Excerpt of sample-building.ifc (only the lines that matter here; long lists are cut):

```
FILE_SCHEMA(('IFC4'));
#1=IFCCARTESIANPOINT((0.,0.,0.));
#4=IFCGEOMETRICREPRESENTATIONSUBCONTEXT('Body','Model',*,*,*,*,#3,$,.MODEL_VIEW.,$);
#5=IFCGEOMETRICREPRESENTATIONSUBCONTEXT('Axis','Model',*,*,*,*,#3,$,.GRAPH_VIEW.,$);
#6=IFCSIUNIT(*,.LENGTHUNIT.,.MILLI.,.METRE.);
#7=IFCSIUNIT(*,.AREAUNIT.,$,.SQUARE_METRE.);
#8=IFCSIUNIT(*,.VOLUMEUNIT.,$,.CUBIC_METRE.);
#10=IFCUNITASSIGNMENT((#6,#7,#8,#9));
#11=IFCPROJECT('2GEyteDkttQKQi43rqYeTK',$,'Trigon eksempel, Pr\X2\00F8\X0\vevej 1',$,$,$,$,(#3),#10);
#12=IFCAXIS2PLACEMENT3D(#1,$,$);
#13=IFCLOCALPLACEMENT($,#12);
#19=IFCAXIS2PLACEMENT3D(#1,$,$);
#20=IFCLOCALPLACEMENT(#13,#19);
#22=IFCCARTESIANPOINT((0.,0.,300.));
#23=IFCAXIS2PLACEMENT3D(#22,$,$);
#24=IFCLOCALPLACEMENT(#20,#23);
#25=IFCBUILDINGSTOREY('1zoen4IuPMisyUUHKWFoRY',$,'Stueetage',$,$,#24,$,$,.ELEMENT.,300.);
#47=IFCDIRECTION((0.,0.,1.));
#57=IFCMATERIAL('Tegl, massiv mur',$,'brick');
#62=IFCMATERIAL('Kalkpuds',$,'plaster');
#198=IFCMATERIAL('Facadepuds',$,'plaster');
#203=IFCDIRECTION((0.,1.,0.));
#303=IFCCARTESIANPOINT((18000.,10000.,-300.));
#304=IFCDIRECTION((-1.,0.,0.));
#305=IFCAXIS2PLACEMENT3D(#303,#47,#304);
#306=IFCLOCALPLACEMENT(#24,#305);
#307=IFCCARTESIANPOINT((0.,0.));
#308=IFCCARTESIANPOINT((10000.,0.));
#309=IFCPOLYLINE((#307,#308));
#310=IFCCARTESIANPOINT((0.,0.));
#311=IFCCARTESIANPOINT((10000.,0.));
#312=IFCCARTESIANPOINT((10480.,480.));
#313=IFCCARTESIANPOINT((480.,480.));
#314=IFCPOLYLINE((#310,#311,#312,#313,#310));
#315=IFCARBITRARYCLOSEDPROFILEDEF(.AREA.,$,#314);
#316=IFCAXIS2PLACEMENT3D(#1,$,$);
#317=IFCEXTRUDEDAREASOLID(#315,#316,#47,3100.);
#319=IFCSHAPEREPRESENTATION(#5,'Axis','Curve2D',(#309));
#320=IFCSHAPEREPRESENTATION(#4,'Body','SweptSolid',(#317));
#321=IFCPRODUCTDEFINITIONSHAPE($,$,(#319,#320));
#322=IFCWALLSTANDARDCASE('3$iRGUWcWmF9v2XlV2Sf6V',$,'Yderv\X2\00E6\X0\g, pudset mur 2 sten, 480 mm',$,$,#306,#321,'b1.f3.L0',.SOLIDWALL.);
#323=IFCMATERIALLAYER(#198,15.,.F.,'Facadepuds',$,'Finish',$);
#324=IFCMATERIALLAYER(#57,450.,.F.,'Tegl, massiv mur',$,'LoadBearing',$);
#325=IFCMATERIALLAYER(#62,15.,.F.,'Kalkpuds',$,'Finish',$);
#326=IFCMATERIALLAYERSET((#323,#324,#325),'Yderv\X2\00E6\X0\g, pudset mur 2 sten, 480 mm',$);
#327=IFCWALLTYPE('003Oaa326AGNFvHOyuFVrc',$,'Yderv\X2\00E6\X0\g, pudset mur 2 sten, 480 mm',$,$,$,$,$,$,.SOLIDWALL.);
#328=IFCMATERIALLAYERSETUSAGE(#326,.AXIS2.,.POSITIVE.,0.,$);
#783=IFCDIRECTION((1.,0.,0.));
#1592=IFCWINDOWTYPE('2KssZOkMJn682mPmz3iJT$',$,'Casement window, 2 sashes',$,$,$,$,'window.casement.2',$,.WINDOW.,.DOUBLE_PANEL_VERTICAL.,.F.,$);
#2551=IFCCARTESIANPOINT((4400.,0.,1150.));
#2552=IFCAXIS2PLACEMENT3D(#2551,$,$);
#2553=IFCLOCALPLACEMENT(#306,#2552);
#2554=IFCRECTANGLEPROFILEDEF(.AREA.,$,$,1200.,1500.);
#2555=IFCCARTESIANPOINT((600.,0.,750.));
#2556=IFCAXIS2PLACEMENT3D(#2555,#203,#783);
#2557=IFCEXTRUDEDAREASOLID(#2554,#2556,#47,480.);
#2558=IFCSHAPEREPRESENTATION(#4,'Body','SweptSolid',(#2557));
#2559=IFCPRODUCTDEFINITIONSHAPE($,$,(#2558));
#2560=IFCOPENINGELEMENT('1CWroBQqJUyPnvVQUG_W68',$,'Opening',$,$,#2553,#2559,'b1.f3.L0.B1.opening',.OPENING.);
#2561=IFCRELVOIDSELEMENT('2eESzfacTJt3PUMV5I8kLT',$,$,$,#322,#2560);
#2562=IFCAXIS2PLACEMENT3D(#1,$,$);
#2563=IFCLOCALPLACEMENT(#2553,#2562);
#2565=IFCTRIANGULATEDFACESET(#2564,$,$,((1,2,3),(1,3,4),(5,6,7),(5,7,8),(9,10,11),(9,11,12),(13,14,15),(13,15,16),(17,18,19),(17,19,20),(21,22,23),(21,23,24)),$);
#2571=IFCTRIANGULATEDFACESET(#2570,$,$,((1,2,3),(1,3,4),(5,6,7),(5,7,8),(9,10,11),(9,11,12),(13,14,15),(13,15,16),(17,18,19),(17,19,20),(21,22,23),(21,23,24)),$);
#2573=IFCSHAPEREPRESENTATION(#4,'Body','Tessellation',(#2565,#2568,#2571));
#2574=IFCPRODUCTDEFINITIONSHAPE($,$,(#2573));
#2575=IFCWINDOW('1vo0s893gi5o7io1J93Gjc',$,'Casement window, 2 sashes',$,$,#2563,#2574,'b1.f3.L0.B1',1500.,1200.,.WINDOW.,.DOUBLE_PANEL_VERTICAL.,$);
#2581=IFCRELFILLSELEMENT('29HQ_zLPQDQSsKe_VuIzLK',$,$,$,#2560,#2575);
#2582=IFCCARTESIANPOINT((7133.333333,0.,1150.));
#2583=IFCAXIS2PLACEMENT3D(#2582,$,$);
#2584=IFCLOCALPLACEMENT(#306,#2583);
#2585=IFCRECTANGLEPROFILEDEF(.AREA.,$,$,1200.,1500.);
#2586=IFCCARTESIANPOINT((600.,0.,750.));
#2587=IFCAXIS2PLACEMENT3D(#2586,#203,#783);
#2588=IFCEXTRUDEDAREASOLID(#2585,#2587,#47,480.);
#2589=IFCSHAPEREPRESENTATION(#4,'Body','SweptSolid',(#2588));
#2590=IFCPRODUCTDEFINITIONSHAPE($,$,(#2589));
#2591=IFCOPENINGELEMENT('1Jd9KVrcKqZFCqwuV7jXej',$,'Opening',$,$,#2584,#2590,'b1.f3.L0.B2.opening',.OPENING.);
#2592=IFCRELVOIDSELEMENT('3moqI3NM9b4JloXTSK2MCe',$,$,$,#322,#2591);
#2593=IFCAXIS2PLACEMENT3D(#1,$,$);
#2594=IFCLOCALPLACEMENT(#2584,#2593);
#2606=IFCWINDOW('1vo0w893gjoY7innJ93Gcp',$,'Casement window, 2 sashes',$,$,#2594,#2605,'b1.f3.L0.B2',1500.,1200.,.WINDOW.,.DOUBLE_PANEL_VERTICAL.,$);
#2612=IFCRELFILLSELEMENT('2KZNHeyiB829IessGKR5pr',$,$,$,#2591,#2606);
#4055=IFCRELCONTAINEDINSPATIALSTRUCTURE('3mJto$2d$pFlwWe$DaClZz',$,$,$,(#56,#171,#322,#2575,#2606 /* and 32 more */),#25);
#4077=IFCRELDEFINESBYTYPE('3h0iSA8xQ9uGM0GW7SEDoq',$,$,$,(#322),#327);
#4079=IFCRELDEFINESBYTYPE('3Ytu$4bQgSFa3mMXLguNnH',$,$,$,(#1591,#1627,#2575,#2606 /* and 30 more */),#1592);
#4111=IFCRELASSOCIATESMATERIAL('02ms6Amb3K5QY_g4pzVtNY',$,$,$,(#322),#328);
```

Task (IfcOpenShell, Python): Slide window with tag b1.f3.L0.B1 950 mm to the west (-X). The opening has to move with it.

```python
import ifcopenshell
import ifcopenshell.api.geometry
import ifcopenshell.util.placement
import ifcopenshell.util.unit

model = ifcopenshell.open("sample-building.ifc")
unit_scale = ifcopenshell.util.unit.calculate_unit_scale(model)

window = model.by_guid("1vo0s893gi5o7io1J93Gjc")
opening = window.FillsVoids[0].RelatingOpeningElement
wall = opening.VoidsElements[0].RelatingBuildingElement

wall_matrix = ifcopenshell.util.placement.get_local_placement(wall.ObjectPlacement)
shift = wall_matrix[:3, 0] * 0.95 / unit_scale
before = ifcopenshell.util.placement.get_local_placement(window.ObjectPlacement)[:3, 3].copy()

# The window is placed relative to its opening, so it follows when the opening moves.
matrix = ifcopenshell.util.placement.get_local_placement(opening.ObjectPlacement)
matrix[:3, 3] += shift
ifcopenshell.api.geometry.edit_object_placement(
    model, product=opening, matrix=matrix, is_si=False, should_transform_children=True
)

after = ifcopenshell.util.placement.get_local_placement(window.ObjectPlacement)[:3, 3]
print("window moved by", (after - before).round(3) + 0.0)

model.write("sample-building-out.ifc")
```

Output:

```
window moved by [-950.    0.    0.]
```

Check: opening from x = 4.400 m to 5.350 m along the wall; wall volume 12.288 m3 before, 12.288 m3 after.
